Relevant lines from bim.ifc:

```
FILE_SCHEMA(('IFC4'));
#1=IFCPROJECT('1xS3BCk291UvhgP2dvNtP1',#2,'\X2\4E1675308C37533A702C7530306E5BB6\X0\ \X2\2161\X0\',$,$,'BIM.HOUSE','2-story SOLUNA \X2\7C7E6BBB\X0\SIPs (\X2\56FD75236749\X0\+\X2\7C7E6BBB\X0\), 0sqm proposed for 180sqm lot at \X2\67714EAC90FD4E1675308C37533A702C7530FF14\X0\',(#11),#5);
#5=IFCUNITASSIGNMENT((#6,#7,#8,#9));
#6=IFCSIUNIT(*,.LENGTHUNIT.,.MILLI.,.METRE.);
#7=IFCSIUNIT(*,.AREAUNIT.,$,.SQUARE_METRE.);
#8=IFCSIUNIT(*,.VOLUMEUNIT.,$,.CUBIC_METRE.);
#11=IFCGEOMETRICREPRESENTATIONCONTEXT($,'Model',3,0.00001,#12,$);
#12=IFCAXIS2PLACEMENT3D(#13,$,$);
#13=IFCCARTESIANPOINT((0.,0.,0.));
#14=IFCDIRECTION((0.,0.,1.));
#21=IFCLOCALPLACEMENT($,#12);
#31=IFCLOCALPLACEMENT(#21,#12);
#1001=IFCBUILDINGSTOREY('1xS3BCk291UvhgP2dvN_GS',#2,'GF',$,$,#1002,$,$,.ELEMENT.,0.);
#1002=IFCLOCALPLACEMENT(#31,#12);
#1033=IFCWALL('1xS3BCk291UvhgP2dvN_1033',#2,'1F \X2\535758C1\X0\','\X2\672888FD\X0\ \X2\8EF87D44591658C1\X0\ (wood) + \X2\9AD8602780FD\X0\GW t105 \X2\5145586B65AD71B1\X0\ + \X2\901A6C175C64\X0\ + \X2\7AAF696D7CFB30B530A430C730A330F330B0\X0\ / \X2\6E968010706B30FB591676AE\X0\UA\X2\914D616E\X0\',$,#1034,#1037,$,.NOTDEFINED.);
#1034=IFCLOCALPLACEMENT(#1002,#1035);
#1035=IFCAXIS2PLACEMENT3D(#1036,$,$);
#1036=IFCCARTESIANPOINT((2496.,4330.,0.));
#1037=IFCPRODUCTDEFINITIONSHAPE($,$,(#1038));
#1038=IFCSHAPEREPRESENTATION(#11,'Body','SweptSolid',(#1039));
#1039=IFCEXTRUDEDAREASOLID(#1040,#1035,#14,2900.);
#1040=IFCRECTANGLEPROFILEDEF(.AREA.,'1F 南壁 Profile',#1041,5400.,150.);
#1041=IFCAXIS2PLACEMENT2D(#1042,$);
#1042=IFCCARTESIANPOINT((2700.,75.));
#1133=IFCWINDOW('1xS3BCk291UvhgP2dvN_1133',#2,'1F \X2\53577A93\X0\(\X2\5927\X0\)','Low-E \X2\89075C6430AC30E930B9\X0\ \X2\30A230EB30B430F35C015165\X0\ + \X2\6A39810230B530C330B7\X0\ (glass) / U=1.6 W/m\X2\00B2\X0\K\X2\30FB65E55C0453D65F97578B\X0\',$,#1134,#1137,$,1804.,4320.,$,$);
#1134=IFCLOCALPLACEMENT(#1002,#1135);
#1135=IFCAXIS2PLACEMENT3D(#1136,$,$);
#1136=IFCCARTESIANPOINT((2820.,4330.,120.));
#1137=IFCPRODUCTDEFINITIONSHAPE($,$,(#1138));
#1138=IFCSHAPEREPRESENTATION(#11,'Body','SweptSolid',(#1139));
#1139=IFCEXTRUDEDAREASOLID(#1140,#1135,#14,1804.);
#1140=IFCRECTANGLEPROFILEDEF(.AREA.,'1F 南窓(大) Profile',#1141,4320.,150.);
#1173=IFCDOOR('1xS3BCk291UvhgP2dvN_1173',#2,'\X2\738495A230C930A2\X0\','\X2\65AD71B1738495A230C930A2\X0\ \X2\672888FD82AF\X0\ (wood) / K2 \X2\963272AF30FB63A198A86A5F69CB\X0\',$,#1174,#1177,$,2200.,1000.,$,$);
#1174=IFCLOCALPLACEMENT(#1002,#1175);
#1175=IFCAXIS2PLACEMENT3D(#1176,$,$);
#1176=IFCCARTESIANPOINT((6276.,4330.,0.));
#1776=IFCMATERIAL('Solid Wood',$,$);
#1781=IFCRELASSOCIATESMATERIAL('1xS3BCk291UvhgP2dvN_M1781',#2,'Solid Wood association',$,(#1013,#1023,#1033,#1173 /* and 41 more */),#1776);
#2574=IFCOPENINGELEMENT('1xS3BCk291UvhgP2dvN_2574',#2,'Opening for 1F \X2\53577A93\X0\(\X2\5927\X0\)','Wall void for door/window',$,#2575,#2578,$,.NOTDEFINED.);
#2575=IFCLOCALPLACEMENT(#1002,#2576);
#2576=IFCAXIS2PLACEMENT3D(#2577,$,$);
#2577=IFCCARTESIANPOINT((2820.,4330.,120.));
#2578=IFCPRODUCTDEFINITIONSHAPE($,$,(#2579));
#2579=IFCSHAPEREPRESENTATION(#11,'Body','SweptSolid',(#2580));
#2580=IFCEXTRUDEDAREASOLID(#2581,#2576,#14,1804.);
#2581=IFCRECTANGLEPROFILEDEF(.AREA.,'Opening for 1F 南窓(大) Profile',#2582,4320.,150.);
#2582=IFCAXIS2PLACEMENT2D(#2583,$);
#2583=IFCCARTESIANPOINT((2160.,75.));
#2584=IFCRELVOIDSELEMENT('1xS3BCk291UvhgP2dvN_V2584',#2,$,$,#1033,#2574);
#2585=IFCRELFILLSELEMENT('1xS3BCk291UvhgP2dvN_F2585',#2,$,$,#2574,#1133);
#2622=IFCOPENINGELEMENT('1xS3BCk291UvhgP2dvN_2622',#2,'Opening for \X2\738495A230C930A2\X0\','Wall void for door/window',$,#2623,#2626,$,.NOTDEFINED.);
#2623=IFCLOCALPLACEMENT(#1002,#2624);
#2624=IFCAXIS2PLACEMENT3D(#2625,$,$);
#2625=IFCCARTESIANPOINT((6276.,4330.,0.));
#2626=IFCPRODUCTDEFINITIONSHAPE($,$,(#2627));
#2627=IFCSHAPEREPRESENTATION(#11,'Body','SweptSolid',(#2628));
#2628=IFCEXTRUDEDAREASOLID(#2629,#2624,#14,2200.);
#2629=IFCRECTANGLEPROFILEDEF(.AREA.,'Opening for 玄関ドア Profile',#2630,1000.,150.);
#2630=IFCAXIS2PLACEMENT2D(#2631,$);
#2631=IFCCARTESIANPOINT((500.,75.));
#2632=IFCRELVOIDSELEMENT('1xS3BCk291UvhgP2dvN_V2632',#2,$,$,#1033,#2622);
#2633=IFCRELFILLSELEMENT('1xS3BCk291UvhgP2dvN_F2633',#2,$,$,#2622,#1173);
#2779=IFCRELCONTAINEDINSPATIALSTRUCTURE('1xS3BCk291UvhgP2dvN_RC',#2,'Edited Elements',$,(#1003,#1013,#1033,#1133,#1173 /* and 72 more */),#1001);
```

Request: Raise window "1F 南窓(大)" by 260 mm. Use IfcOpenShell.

```python
import numpy as np
import ifcopenshell
import ifcopenshell.api.geometry
import ifcopenshell.util.placement
import ifcopenshell.util.unit

model = ifcopenshell.open("bim.ifc")
unit_scale = ifcopenshell.util.unit.calculate_unit_scale(model)

window = model.by_guid("1xS3BCk291UvhgP2dvN_1133")
opening = window.FillsVoids[0].RelatingOpeningElement
dz = 0.26 / unit_scale

shift = np.array([0.0, 0.0, dz])
# The window is not placed relative to its opening, so move both.
for product in (opening, window):
    matrix = ifcopenshell.util.placement.get_local_placement(product.ObjectPlacement)
    matrix[:3, 3] += shift
    ifcopenshell.api.geometry.edit_object_placement(model, product=product, matrix=matrix, is_si=False)

print(f"moved by {dz * unit_scale:+.3f} m")

model.write("bim_rev.ifc")
```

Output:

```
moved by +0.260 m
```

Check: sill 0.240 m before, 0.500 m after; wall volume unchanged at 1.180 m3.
